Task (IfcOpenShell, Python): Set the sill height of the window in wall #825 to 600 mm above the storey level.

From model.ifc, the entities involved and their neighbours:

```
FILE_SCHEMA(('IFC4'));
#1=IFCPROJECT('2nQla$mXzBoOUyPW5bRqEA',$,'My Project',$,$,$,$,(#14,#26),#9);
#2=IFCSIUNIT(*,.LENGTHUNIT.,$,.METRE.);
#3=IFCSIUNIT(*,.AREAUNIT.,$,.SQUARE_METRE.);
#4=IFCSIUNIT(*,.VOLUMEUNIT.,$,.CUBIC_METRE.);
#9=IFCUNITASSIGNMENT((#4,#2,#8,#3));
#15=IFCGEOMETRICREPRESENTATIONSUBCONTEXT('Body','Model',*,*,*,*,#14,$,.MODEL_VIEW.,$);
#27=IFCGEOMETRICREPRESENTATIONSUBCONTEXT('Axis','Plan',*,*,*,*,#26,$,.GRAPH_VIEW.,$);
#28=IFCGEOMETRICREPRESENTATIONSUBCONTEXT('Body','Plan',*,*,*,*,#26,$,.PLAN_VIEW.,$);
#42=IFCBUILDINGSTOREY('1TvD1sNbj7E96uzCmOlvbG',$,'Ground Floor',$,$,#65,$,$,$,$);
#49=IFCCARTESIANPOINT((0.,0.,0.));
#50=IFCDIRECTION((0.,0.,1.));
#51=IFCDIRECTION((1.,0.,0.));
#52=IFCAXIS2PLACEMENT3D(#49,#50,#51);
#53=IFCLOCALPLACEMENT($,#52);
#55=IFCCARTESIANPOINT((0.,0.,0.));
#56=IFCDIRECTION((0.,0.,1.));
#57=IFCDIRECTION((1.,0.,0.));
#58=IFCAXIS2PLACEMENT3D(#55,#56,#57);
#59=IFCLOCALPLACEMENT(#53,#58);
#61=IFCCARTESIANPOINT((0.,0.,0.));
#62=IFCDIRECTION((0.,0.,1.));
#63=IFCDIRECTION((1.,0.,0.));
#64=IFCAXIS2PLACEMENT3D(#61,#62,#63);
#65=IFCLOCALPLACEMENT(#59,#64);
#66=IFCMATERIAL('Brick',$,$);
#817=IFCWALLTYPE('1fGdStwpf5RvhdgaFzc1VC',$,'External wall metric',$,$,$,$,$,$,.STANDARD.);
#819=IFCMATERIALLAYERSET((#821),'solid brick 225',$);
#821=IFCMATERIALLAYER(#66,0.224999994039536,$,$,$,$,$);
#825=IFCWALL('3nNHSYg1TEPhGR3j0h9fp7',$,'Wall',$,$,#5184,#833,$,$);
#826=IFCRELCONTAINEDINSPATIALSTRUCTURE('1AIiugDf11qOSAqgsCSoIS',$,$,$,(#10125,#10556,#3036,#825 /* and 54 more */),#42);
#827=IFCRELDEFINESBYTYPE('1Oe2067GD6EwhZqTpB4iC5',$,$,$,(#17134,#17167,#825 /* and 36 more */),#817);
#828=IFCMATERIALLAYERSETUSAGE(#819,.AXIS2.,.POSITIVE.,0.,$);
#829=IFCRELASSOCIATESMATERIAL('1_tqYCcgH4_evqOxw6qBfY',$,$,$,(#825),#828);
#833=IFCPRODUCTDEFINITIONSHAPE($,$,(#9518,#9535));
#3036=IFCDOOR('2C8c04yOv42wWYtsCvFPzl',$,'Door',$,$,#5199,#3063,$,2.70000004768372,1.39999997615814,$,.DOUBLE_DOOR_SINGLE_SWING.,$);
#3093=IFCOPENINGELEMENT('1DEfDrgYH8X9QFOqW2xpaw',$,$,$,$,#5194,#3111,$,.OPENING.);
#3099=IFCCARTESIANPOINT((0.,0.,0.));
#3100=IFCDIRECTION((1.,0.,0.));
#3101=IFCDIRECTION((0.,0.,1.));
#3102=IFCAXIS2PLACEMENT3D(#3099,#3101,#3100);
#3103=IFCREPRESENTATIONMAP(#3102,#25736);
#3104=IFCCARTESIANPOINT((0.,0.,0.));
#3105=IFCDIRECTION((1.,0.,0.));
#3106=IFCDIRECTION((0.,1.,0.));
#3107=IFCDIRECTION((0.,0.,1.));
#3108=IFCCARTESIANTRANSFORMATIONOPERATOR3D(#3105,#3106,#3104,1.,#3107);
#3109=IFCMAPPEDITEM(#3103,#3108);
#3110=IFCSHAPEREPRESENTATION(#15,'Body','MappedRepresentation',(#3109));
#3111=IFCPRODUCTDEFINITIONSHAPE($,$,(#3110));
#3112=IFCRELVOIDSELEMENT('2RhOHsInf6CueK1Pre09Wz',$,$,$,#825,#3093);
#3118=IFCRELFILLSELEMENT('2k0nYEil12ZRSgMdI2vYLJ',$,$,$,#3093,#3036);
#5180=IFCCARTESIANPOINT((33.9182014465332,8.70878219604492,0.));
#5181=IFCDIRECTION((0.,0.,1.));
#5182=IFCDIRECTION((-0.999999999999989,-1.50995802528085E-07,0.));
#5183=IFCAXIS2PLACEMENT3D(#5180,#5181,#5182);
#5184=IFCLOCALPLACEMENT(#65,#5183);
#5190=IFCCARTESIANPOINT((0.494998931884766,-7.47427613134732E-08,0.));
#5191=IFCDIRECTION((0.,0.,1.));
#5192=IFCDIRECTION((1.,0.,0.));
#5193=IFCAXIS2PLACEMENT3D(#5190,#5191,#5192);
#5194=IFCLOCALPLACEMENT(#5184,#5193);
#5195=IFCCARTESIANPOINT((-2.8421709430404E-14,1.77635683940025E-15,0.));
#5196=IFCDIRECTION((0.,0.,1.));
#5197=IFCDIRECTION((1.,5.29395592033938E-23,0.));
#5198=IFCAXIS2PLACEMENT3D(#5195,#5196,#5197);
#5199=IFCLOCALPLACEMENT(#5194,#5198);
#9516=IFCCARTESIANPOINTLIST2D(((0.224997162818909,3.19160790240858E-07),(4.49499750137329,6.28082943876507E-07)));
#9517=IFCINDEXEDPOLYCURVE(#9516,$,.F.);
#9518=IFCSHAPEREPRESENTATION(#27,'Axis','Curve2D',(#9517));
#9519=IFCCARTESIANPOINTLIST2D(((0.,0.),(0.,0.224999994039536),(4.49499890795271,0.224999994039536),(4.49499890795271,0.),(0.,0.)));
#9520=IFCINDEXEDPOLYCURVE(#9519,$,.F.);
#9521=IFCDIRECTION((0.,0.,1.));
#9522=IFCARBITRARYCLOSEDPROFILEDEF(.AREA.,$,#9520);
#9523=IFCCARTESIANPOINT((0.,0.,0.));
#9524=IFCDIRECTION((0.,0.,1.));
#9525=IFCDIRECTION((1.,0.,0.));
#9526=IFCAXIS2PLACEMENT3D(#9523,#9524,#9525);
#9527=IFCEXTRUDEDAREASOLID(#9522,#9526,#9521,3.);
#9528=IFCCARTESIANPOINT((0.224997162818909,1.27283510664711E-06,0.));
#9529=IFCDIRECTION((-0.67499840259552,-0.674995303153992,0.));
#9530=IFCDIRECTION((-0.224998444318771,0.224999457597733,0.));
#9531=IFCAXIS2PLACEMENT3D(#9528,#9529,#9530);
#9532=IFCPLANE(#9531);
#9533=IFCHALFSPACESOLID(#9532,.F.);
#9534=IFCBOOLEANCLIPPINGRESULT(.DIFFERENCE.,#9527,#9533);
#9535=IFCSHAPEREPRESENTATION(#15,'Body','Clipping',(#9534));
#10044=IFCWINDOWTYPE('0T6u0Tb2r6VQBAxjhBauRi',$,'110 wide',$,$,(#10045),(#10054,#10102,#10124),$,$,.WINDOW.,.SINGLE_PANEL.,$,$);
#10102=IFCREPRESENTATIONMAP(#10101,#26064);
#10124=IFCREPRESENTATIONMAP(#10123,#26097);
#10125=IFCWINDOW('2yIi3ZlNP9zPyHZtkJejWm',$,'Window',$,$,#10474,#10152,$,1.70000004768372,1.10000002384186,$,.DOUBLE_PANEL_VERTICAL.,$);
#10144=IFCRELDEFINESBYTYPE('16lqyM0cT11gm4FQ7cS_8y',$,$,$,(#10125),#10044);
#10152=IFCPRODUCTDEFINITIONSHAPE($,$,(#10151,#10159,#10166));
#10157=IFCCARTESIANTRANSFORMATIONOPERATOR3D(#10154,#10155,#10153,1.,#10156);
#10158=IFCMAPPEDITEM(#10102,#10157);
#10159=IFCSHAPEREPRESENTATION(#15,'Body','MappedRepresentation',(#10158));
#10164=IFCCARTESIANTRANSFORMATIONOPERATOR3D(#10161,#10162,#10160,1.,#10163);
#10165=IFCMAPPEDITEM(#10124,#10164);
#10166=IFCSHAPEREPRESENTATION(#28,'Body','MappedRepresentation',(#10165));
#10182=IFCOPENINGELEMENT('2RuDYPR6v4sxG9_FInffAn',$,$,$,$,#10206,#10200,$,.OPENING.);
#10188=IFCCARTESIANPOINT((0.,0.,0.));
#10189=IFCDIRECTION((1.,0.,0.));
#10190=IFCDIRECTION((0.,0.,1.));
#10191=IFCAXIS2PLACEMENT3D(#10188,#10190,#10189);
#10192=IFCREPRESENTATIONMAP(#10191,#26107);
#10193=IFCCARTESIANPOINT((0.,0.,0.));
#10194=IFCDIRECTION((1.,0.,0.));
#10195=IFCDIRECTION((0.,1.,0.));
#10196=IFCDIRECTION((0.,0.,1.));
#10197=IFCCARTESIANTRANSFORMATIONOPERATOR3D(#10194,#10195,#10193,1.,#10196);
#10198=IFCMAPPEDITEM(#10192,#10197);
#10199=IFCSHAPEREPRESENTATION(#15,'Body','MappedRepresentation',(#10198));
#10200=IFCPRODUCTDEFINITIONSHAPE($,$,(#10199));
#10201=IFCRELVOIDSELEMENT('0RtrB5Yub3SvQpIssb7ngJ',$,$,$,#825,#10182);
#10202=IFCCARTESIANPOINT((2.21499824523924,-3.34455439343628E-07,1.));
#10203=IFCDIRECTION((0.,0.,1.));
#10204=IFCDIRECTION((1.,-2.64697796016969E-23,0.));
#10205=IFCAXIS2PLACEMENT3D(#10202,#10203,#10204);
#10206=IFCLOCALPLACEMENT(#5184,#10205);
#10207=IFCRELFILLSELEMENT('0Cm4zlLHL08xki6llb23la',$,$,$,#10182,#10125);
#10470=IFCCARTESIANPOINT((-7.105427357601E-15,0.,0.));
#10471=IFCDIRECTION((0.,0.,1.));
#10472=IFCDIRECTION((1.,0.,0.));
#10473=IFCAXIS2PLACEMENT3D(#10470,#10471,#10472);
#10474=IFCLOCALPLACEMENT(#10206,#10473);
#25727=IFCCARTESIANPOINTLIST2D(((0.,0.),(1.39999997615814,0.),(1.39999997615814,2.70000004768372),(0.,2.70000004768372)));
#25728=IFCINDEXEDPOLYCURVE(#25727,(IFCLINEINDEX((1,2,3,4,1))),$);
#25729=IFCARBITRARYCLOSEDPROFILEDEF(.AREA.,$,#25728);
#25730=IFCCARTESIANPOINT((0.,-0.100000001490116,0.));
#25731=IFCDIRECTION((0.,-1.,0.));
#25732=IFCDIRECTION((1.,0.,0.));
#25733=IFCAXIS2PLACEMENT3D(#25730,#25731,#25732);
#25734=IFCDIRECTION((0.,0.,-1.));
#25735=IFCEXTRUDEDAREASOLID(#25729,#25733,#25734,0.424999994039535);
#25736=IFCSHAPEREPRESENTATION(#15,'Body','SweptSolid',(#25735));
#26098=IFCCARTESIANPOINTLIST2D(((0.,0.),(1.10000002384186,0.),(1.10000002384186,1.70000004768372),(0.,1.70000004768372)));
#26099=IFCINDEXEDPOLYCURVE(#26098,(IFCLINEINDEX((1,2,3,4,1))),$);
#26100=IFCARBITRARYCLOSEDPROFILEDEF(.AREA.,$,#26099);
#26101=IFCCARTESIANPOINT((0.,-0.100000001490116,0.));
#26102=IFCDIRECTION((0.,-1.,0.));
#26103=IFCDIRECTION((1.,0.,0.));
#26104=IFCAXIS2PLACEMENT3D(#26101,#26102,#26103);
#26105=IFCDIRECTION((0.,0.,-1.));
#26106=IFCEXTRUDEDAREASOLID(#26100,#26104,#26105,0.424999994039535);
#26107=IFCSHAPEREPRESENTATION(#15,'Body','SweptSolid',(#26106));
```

```python
import numpy as np
import ifcopenshell
import ifcopenshell.api.geometry
import ifcopenshell.geom
import ifcopenshell.util.element
import ifcopenshell.util.placement
import ifcopenshell.util.shape
import ifcopenshell.util.unit

model = ifcopenshell.open("model.ifc")
unit_scale = ifcopenshell.util.unit.calculate_unit_scale(model)

window = model.by_guid("2yIi3ZlNP9zPyHZtkJejWm")
opening = window.FillsVoids[0].RelatingOpeningElement
storey = ifcopenshell.util.element.get_container(window, ifc_class="IfcBuildingStorey")
level = ifcopenshell.util.placement.get_local_placement(storey.ObjectPlacement)[2, 3]

# The opening's origin need not be at the sill, so measure its lowest point.
shape = ifcopenshell.geom.create_shape(ifcopenshell.geom.settings(), opening)
bottom = ifcopenshell.util.shape.get_shape_bottom_elevation(shape, shape.geometry) / unit_scale
dz = level + 0.6 - bottom

shift = np.array([0.0, 0.0, dz])
# The window is placed relative to its opening, so it follows when the opening moves.
matrix = ifcopenshell.util.placement.get_local_placement(opening.ObjectPlacement)
matrix[:3, 3] += shift
ifcopenshell.api.geometry.edit_object_placement(
    model, product=opening, matrix=matrix, is_si=False, should_transform_children=True
)

print(f"moved by {dz * unit_scale:+.3f} m")

model.write("model_rev.ifc")
```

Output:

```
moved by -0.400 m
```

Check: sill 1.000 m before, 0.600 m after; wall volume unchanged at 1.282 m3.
